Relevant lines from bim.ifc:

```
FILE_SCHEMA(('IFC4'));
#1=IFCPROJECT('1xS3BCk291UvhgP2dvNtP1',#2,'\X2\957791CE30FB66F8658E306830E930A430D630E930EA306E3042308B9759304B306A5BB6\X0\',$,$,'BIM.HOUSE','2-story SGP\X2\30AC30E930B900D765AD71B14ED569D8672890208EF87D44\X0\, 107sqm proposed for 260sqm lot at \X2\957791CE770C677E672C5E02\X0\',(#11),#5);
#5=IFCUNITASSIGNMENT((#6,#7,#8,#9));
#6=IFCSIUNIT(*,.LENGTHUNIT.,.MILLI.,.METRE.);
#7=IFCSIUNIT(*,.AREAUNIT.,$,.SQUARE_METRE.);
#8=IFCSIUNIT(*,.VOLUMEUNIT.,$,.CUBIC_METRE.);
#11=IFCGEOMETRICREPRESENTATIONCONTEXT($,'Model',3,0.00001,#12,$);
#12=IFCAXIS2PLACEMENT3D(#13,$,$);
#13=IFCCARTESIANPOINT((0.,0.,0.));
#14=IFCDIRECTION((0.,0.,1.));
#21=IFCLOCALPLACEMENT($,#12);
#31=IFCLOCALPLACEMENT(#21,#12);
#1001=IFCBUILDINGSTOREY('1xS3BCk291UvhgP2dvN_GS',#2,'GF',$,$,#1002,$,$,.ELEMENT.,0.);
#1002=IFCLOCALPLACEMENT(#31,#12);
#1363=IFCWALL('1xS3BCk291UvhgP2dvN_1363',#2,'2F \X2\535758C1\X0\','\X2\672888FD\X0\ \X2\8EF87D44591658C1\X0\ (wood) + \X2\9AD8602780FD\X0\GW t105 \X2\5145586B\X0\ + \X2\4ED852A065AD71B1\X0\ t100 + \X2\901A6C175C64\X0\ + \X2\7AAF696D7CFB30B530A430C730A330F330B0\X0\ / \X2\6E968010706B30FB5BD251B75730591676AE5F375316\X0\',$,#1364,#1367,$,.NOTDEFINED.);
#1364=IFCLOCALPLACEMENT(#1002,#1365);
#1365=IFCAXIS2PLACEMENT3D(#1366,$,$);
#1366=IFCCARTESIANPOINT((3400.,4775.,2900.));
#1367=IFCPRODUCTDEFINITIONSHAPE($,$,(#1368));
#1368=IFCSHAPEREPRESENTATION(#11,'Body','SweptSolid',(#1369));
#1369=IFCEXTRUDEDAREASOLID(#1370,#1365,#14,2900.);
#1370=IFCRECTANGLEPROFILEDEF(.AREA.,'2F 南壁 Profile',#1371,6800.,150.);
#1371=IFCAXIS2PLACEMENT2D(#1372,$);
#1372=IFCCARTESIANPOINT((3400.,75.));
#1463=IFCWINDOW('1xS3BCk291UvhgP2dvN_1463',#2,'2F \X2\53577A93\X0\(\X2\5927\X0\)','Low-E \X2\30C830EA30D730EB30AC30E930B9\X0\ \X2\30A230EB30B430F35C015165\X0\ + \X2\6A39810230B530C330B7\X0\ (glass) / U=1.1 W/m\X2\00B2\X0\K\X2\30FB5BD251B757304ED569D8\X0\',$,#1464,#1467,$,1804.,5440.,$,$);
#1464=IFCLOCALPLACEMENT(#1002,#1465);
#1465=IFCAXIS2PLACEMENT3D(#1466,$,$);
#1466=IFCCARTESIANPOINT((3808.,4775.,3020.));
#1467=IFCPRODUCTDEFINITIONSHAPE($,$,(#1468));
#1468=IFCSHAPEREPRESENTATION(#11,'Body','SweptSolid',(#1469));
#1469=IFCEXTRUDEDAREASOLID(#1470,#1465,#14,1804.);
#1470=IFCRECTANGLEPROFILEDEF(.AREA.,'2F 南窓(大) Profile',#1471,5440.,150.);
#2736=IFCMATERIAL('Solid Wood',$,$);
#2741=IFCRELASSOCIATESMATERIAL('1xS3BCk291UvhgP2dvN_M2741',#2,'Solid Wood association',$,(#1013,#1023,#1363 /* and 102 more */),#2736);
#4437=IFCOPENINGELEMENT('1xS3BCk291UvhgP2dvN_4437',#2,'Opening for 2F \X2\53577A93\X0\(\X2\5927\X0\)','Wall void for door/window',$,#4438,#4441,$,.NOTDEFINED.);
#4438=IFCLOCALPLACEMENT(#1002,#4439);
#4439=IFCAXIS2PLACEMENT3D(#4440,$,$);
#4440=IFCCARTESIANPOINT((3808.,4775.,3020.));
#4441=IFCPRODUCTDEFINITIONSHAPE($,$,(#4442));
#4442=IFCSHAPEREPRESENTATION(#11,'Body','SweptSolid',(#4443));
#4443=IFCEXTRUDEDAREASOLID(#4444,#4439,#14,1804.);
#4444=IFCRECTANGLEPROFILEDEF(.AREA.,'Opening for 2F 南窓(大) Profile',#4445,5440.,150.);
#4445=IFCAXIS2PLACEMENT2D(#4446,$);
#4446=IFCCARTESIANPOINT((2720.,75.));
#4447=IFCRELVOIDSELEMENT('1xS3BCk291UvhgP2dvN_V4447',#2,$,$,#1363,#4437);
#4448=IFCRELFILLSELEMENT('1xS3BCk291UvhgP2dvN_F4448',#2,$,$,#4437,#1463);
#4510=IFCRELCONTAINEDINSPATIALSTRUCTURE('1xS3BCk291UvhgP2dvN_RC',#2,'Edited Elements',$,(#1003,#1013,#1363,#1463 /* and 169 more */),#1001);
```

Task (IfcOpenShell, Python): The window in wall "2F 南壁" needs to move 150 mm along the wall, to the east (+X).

```python
import ifcopenshell
import ifcopenshell.api.geometry
import ifcopenshell.util.placement
import ifcopenshell.util.unit

model = ifcopenshell.open("bim.ifc")
unit_scale = ifcopenshell.util.unit.calculate_unit_scale(model)

window = model.by_guid("1xS3BCk291UvhgP2dvN_1463")
opening = window.FillsVoids[0].RelatingOpeningElement
wall = opening.VoidsElements[0].RelatingBuildingElement

wall_matrix = ifcopenshell.util.placement.get_local_placement(wall.ObjectPlacement)
shift = wall_matrix[:3, 0] * 0.15 / unit_scale
before = ifcopenshell.util.placement.get_local_placement(window.ObjectPlacement)[:3, 3].copy()

# The window is not placed relative to its opening, so move both.
for product in (opening, window):
    matrix = ifcopenshell.util.placement.get_local_placement(product.ObjectPlacement)
    matrix[:3, 3] += shift
    ifcopenshell.api.geometry.edit_object_placement(model, product=product, matrix=matrix, is_si=False)

after = ifcopenshell.util.placement.get_local_placement(window.ObjectPlacement)[:3, 3]
print("window moved by", (after - before).round(3) + 0.0)

model.write("bim_rev.ifc")
```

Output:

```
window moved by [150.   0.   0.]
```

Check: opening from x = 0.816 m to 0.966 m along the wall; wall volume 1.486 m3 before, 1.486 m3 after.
